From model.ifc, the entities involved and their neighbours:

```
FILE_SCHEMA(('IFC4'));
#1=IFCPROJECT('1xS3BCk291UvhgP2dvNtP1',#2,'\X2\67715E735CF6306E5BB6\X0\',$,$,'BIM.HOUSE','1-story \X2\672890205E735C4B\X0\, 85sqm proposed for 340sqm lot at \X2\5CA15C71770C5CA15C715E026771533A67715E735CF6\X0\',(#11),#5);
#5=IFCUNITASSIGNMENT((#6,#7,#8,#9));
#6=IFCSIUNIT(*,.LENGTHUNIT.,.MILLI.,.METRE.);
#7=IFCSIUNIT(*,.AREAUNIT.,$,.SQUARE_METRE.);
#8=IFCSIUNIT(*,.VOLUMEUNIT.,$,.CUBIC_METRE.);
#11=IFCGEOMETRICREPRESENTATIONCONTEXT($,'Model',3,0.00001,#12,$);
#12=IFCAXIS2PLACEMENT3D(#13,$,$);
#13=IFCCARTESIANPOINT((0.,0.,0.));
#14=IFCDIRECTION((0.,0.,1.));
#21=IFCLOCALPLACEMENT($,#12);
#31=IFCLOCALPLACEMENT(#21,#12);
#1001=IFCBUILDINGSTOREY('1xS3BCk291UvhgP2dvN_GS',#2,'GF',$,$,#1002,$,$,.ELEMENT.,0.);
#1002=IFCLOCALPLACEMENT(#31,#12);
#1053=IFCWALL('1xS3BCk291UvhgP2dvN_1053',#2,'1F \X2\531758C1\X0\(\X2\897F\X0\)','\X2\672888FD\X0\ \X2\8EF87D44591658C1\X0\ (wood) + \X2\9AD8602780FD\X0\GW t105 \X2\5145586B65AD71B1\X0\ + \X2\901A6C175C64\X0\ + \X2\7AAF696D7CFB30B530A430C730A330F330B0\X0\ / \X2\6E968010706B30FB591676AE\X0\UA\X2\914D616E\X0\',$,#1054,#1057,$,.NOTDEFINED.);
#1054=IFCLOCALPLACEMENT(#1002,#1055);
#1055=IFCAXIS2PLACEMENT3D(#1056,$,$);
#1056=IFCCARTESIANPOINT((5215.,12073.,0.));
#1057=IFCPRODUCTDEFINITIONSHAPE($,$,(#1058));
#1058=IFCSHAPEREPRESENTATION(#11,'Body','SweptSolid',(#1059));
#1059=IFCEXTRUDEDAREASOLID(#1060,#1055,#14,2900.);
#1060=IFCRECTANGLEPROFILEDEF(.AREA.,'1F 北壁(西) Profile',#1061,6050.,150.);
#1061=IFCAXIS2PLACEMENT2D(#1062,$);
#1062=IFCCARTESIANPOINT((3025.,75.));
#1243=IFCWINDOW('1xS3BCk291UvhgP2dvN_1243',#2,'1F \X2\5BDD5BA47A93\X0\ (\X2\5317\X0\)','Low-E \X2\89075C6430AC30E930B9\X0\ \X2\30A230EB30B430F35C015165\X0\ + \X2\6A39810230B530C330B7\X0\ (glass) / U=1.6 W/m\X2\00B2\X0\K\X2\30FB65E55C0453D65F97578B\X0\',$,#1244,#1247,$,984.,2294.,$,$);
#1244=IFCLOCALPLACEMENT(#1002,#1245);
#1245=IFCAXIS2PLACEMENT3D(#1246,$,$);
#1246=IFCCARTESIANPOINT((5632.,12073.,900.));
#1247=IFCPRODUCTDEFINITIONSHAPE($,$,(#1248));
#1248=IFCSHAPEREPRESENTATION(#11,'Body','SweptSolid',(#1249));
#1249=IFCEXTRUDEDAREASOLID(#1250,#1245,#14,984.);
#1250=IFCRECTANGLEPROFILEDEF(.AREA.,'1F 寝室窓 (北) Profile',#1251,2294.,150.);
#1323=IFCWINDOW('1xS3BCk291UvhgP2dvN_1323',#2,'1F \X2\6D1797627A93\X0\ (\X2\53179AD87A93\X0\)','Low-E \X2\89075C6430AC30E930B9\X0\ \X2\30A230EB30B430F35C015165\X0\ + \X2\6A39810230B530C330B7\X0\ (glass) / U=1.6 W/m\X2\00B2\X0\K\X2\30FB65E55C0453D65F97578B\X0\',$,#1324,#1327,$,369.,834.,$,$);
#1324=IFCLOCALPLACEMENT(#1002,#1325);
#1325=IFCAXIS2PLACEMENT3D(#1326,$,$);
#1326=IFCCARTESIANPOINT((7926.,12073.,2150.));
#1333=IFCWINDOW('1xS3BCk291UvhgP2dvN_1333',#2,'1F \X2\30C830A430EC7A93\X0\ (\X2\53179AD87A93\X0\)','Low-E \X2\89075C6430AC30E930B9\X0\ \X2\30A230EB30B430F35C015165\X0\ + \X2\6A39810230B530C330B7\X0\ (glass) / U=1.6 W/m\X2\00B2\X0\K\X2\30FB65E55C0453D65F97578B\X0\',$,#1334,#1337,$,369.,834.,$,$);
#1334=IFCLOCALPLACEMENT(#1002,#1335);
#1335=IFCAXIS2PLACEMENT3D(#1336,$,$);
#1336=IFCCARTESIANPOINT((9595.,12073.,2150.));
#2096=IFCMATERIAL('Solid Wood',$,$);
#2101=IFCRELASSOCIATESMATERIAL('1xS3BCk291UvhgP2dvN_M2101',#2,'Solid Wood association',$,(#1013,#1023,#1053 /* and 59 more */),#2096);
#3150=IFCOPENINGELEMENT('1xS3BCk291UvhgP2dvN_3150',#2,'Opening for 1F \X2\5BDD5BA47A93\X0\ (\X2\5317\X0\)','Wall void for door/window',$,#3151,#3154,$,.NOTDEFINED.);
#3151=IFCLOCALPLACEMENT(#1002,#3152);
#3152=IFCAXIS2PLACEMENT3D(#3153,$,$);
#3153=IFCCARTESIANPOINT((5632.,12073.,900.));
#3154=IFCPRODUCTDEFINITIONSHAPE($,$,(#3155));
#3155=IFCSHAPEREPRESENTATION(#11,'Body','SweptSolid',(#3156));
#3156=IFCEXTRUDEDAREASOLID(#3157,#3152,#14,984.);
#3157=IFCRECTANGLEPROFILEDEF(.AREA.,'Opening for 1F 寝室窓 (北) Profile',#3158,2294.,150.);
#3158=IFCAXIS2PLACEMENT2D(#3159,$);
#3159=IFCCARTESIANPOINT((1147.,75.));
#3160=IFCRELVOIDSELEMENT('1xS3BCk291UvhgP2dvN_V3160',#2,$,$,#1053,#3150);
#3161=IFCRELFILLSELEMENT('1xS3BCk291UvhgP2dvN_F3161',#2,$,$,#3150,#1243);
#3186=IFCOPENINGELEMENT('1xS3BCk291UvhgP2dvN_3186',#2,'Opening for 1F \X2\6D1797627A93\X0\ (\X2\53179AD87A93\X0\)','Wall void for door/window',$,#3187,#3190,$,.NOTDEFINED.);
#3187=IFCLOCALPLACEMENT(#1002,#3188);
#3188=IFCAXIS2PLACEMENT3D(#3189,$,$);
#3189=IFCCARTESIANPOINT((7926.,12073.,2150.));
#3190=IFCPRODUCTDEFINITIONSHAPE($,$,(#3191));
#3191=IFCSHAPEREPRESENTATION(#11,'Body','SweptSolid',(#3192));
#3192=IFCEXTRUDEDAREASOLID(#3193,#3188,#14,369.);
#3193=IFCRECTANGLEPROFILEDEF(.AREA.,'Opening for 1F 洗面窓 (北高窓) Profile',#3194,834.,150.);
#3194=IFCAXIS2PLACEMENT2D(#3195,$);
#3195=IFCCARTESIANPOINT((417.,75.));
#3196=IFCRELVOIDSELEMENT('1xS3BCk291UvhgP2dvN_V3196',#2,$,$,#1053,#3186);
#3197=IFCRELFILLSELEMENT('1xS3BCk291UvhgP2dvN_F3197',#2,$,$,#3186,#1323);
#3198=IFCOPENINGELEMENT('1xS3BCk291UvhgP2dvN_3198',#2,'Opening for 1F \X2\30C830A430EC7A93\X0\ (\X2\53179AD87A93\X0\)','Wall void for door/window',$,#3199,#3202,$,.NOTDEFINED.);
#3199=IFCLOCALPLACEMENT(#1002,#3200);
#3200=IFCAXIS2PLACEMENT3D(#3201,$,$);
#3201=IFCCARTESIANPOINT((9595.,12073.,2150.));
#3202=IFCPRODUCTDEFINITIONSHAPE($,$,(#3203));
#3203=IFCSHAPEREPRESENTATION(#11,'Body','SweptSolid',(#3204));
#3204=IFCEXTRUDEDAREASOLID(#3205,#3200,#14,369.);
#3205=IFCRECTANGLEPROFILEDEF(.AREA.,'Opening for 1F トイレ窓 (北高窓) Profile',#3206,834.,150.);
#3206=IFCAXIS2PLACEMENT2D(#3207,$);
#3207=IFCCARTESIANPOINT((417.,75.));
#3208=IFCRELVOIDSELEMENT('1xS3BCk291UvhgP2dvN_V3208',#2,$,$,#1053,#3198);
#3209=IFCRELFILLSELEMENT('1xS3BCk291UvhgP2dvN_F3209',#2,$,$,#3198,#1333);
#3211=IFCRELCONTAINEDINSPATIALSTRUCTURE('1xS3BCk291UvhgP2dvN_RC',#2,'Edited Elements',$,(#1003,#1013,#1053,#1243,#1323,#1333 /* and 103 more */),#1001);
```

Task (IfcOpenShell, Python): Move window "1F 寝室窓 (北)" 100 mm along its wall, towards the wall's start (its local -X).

```python
import ifcopenshell
import ifcopenshell.api.geometry
import ifcopenshell.util.placement
import ifcopenshell.util.unit

model = ifcopenshell.open("model.ifc")
unit_scale = ifcopenshell.util.unit.calculate_unit_scale(model)

window = model.by_guid("1xS3BCk291UvhgP2dvN_1243")
opening = window.FillsVoids[0].RelatingOpeningElement
wall = opening.VoidsElements[0].RelatingBuildingElement

wall_matrix = ifcopenshell.util.placement.get_local_placement(wall.ObjectPlacement)
shift = wall_matrix[:3, 0] * -0.1 / unit_scale
before = ifcopenshell.util.placement.get_local_placement(window.ObjectPlacement)[:3, 3].copy()

# The window is not placed relative to its opening, so move both.
for product in (opening, window):
    matrix = ifcopenshell.util.placement.get_local_placement(product.ObjectPlacement)
    matrix[:3, 3] += shift
    ifcopenshell.api.geometry.edit_object_placement(model, product=product, matrix=matrix, is_si=False)

after = ifcopenshell.util.placement.get_local_placement(window.ObjectPlacement)[:3, 3]
print("window moved by", (after - before).round(3) + 0.0)

model.write("model_v2.ifc")
```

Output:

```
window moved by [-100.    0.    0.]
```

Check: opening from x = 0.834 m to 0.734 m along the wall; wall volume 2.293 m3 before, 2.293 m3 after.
